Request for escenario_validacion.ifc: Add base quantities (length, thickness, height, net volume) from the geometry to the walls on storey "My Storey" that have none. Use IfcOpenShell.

First a look at what the model holds.

```python
import ifcopenshell
import ifcopenshell.util.element
import ifcopenshell.util.unit

model = ifcopenshell.open("escenario_validacion.ifc")
print(model.schema)
for unit_type in ("LENGTHUNIT", "AREAUNIT", "VOLUMEUNIT"):
    print(unit_type, ifcopenshell.util.unit.calculate_unit_scale(model, unit_type))
storey = next(s for s in model.by_type("IfcBuildingStorey") if s.Name == "My Storey")
walls = [e for e in ifcopenshell.util.element.get_decomposition(storey) if e.is_a("IfcWall")]
for e in sorted(walls, key=lambda e: e.id()):
    print(e.id(), e.is_a(), e.Name, list(ifcopenshell.util.element.get_psets(e, qtos_only=True)), sep=" | ")
```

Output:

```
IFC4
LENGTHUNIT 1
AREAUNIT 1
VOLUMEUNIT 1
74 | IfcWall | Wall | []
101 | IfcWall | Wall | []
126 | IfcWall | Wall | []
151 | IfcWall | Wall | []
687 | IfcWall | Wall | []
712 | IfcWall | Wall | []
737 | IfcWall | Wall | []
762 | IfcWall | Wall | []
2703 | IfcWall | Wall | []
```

```python
import ifcopenshell
import ifcopenshell.api.pset
import ifcopenshell.geom
import ifcopenshell.util.element
import ifcopenshell.util.shape
import ifcopenshell.util.unit

model = ifcopenshell.open("escenario_validacion.ifc")
unit_scale = ifcopenshell.util.unit.calculate_unit_scale(model)
volume_scale = ifcopenshell.util.unit.calculate_unit_scale(model, "VOLUMEUNIT")
settings = ifcopenshell.geom.settings()

storey = next(s for s in model.by_type("IfcBuildingStorey") if s.Name == "My Storey")
walls = [e for e in ifcopenshell.util.element.get_decomposition(storey) if e.is_a("IfcWall")]

for e in sorted(walls, key=lambda e: e.id()):
    if ifcopenshell.util.element.get_psets(e, qtos_only=True, should_inherit=False):
        continue
    # Geometry comes back in metres, in the element's own axes.
    shape = ifcopenshell.geom.create_shape(settings, e)
    values = {
        "Length": ifcopenshell.util.shape.get_x(shape.geometry) / unit_scale,
        "Width": ifcopenshell.util.shape.get_y(shape.geometry) / unit_scale,
        "Height": ifcopenshell.util.shape.get_z(shape.geometry) / unit_scale,
        "NetVolume": ifcopenshell.util.shape.get_volume(shape.geometry) / volume_scale,
    }
    qto = ifcopenshell.api.pset.add_qto(model, product=e, name="Qto_WallBaseQuantities")
    ifcopenshell.api.pset.edit_qto(model, qto=qto, properties=values)
    print(e.id(), {k: round(v, 3) for k, v in values.items()})

model.write("escenario_validacion_rev.ifc")
```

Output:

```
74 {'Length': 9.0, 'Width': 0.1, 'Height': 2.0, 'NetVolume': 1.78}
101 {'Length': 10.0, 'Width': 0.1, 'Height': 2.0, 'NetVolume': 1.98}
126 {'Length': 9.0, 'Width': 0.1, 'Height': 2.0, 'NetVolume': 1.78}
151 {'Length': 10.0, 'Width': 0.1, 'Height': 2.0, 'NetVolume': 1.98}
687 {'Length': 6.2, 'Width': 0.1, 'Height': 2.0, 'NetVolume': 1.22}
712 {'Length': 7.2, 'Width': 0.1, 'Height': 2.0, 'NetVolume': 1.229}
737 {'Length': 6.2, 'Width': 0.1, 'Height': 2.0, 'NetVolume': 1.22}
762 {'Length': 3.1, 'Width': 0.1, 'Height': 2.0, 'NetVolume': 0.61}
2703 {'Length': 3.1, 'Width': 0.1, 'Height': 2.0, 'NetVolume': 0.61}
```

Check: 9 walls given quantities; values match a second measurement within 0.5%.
